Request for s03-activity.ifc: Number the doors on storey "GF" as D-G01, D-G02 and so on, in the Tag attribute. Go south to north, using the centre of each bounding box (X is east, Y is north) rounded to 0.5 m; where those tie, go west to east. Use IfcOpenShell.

First a look at what the model holds.

```python
import ifcopenshell
import ifcopenshell.util.element
import ifcopenshell.util.placement

model = ifcopenshell.open("s03-activity.ifc")
print(model.schema)
storey = next(s for s in model.by_type("IfcBuildingStorey") if s.Name == "GF")
doors = [e for e in ifcopenshell.util.element.get_decomposition(storey) if e.is_a("IfcDoor")]
for e in sorted(doors, key=lambda e: e.id()):
    origin = ifcopenshell.util.placement.get_local_placement(e.ObjectPlacement)[:3, 3]
    print(e.id(), e.Tag, e.Name, origin.round(2) + 0.0, sep=" | ")
```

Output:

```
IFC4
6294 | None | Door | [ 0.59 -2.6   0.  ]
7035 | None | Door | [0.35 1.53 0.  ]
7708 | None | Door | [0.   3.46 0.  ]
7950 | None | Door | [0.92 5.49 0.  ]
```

```python
import ifcopenshell
import ifcopenshell.geom
import ifcopenshell.util.element
import ifcopenshell.util.shape

model = ifcopenshell.open("s03-activity.ifc")
settings = ifcopenshell.geom.settings()
settings.set("use-world-coords", True)


def centre(element):
    shape = ifcopenshell.geom.create_shape(settings, element)
    return ifcopenshell.util.shape.get_bbox_centroid(shape.geometry)


storey = next(s for s in model.by_type("IfcBuildingStorey") if s.Name == "GF")
doors = [e for e in ifcopenshell.util.element.get_decomposition(storey) if e.is_a("IfcDoor")]

# Insertion points can sit at a corner or the storey origin, so sort by the geometry (in metres).
centres = {e: centre(e) for e in doors}
doors.sort(key=lambda e: (round(centres[e][1] / 0.5), centres[e][0]))

for i, e in enumerate(doors, start=1):
    number = f"D-G{i:02d}"
    e.Tag = number
    print(e.id(), number)

model.write("s03-activity_rev.ifc")
```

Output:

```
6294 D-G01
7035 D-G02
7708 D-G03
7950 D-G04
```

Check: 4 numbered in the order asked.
